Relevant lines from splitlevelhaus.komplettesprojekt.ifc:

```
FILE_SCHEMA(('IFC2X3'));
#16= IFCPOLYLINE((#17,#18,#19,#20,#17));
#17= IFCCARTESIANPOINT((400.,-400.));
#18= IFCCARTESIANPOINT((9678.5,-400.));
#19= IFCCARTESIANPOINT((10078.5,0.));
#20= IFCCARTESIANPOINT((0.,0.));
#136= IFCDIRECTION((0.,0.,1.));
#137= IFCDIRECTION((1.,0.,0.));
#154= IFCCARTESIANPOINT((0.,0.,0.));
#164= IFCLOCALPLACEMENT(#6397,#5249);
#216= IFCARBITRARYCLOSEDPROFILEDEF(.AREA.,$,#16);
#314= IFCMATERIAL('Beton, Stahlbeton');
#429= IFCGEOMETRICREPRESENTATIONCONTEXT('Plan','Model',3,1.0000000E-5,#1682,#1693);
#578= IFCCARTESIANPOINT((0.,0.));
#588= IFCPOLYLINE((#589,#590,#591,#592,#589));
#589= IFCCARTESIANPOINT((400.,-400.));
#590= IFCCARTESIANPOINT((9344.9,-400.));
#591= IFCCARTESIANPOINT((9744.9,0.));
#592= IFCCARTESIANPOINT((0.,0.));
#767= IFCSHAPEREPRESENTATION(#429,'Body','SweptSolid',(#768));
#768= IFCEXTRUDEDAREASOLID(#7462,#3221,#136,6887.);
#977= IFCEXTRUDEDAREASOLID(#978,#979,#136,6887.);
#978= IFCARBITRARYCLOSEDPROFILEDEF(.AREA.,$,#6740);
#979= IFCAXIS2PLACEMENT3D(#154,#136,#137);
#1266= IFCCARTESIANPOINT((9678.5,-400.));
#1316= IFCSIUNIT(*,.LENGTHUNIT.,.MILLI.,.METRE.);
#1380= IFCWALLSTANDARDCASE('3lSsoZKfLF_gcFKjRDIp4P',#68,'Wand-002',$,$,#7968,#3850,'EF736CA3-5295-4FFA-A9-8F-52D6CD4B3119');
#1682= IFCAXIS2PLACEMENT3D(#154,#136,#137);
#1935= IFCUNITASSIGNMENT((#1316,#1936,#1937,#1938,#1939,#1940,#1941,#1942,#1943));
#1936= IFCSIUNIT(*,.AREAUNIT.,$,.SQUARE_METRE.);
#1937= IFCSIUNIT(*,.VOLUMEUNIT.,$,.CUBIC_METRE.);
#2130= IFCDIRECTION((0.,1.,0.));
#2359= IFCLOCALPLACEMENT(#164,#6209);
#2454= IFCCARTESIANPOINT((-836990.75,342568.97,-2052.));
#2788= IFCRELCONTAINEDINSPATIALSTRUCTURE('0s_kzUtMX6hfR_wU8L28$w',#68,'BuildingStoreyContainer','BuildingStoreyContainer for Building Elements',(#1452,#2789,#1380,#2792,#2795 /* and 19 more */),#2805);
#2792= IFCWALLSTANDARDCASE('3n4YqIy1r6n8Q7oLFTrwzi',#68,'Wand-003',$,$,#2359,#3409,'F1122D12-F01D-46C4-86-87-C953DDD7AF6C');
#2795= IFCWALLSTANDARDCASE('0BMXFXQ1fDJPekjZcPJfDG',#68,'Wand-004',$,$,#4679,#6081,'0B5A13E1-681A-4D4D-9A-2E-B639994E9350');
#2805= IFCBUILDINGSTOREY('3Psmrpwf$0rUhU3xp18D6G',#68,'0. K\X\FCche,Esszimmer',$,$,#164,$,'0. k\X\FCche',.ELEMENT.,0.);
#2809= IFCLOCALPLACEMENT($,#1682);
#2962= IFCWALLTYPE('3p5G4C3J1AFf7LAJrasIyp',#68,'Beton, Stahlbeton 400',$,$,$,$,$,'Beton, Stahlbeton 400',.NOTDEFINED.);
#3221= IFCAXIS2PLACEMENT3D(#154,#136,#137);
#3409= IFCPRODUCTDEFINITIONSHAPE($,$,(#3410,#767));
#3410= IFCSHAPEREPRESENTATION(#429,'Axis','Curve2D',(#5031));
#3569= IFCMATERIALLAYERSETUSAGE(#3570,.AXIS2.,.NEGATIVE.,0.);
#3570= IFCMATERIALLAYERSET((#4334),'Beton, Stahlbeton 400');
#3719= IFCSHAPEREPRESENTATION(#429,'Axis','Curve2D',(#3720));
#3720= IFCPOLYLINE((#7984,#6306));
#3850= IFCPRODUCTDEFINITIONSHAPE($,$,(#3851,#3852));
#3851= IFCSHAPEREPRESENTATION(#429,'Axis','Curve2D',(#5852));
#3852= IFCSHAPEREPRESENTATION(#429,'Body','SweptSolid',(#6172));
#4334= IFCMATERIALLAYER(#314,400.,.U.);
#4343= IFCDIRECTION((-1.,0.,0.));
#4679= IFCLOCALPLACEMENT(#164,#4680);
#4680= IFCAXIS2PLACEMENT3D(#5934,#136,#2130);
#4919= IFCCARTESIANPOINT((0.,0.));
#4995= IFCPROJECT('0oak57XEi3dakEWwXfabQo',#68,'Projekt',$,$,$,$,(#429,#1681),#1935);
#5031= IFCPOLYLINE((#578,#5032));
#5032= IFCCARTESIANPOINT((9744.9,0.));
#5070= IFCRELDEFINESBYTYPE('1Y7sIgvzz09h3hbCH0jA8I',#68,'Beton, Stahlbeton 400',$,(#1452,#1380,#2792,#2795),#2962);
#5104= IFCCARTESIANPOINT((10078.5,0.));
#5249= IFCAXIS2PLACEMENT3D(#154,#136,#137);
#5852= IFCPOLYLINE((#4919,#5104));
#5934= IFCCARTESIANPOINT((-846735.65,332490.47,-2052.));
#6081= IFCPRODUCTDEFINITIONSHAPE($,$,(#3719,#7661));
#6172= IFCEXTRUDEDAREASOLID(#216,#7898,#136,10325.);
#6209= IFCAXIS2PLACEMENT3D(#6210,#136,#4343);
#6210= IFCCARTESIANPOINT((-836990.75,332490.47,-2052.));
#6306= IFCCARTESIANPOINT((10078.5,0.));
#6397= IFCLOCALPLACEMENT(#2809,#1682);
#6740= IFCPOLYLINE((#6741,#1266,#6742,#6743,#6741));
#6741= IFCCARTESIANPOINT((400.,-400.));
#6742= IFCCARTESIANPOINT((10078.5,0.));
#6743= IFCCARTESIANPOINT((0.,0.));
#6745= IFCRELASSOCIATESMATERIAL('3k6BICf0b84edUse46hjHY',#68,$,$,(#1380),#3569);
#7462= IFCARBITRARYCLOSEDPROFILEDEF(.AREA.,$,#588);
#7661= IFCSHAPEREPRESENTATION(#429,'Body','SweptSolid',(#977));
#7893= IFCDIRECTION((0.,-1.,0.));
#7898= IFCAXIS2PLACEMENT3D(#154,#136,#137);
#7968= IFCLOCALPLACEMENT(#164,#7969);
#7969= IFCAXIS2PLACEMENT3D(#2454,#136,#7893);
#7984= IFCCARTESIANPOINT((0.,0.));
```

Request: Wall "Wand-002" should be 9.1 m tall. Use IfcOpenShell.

```python
import ifcopenshell
import ifcopenshell.geom
import ifcopenshell.util.shape

model = ifcopenshell.open("splitlevelhaus.komplettesprojekt.ifc")
settings = ifcopenshell.geom.settings()


def volume(element):
    """Net volume in cubic metres, openings subtracted."""
    shape = ifcopenshell.geom.create_shape(settings, element)
    return ifcopenshell.util.shape.get_volume(shape.geometry)


wall = model.by_guid("3lSsoZKfLF_gcFKjRDIp4P")
before = volume(wall)

body = next(r for r in wall.Representation.Representations if r.RepresentationIdentifier == "Body")
solid = body.Items[0]
old_height = solid.Depth
solid.Depth = 9100.0
after = volume(wall)

print(f"height {old_height:g} -> {solid.Depth:g}, volume {before:.3f} -> {after:.3f} m3")

model.write("splitlevelhaus.komplettesprojekt_edited.ifc")
```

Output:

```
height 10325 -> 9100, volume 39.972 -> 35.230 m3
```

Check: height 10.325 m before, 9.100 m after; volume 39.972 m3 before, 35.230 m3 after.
